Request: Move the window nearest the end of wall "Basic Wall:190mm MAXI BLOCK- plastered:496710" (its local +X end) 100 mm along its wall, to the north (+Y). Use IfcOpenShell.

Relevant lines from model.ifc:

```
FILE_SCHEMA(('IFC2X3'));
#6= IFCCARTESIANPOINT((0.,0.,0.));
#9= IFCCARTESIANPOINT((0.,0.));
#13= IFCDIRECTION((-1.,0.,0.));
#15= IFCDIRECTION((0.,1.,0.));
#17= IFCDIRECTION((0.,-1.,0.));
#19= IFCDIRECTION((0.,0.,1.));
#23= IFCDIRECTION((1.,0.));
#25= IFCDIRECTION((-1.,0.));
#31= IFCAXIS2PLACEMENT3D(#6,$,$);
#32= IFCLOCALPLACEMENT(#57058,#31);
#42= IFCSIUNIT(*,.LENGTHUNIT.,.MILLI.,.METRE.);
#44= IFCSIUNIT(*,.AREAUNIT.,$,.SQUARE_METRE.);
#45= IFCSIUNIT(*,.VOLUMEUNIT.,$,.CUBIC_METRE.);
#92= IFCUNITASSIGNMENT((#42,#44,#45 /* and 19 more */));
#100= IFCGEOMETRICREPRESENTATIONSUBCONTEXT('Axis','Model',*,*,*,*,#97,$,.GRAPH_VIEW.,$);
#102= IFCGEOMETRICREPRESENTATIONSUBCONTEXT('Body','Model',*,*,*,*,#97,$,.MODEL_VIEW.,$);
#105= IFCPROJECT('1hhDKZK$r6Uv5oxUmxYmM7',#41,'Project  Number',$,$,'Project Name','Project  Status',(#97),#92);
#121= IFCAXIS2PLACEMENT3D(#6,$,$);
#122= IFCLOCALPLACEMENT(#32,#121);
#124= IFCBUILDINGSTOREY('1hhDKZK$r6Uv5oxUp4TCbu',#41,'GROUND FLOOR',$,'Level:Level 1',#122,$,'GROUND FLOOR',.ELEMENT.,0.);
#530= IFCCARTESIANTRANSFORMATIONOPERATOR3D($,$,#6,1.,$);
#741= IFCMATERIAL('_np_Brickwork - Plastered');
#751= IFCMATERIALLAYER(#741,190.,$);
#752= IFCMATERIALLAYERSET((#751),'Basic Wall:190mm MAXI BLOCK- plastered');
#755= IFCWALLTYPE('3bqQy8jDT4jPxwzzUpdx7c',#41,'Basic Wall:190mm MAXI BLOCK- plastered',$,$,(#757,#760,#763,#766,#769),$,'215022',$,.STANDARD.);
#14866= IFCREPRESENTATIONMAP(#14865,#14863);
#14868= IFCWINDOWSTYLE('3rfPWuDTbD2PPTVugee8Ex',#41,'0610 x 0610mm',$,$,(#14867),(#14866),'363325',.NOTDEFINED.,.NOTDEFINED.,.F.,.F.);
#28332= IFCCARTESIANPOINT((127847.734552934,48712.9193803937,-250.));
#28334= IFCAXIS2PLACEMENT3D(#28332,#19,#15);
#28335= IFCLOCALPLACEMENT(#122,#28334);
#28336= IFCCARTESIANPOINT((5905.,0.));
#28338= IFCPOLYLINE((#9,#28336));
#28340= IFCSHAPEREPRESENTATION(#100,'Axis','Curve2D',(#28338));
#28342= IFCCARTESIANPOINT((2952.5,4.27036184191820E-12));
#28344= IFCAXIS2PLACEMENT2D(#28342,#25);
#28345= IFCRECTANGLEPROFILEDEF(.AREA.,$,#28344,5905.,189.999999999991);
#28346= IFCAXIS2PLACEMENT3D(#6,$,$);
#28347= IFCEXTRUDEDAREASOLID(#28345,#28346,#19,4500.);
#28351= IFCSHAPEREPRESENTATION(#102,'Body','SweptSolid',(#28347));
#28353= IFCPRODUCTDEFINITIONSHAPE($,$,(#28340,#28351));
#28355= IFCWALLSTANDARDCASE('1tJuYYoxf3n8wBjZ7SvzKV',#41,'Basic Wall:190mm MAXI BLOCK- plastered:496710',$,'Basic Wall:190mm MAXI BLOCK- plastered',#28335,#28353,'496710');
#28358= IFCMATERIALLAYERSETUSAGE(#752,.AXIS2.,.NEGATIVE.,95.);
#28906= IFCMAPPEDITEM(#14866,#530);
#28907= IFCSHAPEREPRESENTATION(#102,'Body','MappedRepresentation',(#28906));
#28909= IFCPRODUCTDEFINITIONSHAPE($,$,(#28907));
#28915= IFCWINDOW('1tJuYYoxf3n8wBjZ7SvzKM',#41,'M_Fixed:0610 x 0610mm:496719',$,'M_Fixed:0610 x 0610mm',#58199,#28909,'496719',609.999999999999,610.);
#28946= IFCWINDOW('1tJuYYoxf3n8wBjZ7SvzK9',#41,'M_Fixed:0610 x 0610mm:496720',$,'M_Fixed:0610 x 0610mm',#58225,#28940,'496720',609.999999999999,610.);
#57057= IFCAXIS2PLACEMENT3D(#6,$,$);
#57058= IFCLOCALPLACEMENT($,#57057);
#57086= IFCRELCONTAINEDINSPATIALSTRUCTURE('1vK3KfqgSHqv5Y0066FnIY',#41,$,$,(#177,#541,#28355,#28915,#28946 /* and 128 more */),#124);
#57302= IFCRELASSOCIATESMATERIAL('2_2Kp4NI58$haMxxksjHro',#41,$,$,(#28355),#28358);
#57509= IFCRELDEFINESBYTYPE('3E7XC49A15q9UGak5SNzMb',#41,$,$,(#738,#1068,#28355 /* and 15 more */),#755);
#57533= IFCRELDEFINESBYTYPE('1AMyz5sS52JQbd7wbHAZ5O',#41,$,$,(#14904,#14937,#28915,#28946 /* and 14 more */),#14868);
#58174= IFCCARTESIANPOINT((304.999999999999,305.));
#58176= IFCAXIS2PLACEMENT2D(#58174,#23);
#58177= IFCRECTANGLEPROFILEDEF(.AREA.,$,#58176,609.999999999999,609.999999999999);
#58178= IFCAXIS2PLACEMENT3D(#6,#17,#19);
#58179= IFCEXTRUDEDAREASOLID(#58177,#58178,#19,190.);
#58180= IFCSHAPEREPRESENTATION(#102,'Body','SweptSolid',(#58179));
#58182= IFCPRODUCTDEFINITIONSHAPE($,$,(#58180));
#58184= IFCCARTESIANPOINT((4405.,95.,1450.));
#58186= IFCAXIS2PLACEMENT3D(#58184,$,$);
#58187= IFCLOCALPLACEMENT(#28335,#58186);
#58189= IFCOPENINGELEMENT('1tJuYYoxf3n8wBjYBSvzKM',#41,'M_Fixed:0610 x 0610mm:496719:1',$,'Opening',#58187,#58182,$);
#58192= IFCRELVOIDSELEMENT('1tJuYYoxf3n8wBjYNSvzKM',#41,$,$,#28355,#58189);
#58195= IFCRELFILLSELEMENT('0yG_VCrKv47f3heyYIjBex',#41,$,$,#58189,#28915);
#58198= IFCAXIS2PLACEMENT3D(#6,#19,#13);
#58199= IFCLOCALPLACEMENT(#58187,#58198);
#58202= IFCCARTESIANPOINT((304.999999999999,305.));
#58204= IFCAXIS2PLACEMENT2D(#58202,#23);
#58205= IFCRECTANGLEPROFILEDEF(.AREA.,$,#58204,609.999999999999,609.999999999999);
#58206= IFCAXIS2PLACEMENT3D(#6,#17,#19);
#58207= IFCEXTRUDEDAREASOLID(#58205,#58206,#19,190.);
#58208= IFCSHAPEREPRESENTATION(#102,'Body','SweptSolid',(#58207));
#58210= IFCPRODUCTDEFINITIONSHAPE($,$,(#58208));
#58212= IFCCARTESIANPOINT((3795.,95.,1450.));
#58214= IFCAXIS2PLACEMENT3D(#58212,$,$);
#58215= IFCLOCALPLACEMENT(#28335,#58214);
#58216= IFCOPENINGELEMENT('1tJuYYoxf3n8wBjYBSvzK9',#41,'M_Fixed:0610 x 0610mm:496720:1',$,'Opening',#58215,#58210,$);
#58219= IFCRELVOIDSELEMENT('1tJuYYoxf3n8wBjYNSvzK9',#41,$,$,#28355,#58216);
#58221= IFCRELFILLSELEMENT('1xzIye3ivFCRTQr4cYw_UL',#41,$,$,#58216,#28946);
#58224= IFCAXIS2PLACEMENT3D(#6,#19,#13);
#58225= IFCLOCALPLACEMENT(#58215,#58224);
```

```python
import ifcopenshell
import ifcopenshell.api.geometry
import ifcopenshell.util.placement
import ifcopenshell.util.unit

model = ifcopenshell.open("model.ifc")
unit_scale = ifcopenshell.util.unit.calculate_unit_scale(model)

window = model.by_guid("1tJuYYoxf3n8wBjZ7SvzKM")
opening = window.FillsVoids[0].RelatingOpeningElement
wall = opening.VoidsElements[0].RelatingBuildingElement

wall_matrix = ifcopenshell.util.placement.get_local_placement(wall.ObjectPlacement)
shift = wall_matrix[:3, 0] * 0.1 / unit_scale
before = ifcopenshell.util.placement.get_local_placement(window.ObjectPlacement)[:3, 3].copy()

# The window is placed relative to its opening, so it follows when the opening moves.
matrix = ifcopenshell.util.placement.get_local_placement(opening.ObjectPlacement)
matrix[:3, 3] += shift
ifcopenshell.api.geometry.edit_object_placement(
    model, product=opening, matrix=matrix, is_si=False, should_transform_children=True
)

after = ifcopenshell.util.placement.get_local_placement(window.ObjectPlacement)[:3, 3]
print("window moved by", (after - before).round(3) + 0.0)

model.write("model_edited.ifc")
```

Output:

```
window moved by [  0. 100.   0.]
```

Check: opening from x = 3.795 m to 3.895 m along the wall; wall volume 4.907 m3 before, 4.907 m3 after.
